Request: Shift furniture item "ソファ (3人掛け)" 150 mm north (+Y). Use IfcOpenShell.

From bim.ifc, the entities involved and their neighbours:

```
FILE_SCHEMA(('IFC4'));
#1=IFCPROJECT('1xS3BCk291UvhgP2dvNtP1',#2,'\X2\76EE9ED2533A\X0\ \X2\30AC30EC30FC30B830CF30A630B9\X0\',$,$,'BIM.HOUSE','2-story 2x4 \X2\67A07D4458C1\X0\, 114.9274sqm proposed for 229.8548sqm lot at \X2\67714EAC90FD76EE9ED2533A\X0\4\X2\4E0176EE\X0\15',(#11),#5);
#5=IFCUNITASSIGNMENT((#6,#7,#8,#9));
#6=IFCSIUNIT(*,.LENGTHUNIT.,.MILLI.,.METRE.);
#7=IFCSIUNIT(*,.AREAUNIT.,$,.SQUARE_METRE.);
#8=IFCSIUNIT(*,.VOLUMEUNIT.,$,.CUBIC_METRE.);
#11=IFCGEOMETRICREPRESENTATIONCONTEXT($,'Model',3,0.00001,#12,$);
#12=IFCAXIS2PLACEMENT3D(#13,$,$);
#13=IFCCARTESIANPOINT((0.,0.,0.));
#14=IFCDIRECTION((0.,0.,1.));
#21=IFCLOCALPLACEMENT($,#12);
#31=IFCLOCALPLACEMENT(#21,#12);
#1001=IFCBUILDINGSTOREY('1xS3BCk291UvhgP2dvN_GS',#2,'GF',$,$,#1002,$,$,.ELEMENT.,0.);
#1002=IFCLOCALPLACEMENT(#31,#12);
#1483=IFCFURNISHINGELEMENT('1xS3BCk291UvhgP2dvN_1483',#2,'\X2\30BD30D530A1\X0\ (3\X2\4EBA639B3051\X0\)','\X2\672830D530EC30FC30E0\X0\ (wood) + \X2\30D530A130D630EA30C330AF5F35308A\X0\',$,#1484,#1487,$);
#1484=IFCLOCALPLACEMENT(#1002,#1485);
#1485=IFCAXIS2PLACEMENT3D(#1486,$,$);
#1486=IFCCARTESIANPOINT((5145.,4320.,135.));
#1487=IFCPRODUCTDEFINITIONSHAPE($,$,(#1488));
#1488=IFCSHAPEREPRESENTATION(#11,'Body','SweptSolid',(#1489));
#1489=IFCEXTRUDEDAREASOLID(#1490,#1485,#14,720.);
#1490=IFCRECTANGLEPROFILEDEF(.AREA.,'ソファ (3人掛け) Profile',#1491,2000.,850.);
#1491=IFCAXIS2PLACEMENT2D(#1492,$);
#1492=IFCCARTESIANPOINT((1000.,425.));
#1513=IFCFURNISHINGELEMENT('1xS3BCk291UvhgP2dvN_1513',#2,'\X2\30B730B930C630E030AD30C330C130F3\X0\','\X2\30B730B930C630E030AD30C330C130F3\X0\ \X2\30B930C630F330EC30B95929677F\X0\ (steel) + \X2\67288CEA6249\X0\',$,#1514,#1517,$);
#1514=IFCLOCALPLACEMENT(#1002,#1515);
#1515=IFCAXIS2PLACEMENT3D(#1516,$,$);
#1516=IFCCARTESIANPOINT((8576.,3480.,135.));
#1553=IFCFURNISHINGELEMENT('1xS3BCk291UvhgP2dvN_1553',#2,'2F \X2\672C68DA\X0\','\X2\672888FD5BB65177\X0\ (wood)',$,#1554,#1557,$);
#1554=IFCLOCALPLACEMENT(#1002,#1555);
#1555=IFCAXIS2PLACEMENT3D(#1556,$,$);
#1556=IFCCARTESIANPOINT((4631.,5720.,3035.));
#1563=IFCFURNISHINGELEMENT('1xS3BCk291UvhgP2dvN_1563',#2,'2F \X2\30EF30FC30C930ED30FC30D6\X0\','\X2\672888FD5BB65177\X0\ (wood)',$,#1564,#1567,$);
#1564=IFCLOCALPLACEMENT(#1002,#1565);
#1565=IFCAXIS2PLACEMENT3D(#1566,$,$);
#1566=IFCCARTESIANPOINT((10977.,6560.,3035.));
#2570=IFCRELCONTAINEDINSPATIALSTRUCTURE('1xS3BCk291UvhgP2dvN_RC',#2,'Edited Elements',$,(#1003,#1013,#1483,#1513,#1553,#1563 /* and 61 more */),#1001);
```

```python
import ifcopenshell
import ifcopenshell.api.geometry
import ifcopenshell.util.placement
import ifcopenshell.util.unit

model = ifcopenshell.open("bim.ifc")
unit_scale = ifcopenshell.util.unit.calculate_unit_scale(model)

item = model.by_guid("1xS3BCk291UvhgP2dvN_1483")
matrix = ifcopenshell.util.placement.get_local_placement(item.ObjectPlacement)
matrix[1, 3] += 0.15 / unit_scale
ifcopenshell.api.geometry.edit_object_placement(model, product=item, matrix=matrix, is_si=False)

print(ifcopenshell.util.placement.get_local_placement(item.ObjectPlacement).round(3) + 0.0)

model.write("bim-out.ifc")
```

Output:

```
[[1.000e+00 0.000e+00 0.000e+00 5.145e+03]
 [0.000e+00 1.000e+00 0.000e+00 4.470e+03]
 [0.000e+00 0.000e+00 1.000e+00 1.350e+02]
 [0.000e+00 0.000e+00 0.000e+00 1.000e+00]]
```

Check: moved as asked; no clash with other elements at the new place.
